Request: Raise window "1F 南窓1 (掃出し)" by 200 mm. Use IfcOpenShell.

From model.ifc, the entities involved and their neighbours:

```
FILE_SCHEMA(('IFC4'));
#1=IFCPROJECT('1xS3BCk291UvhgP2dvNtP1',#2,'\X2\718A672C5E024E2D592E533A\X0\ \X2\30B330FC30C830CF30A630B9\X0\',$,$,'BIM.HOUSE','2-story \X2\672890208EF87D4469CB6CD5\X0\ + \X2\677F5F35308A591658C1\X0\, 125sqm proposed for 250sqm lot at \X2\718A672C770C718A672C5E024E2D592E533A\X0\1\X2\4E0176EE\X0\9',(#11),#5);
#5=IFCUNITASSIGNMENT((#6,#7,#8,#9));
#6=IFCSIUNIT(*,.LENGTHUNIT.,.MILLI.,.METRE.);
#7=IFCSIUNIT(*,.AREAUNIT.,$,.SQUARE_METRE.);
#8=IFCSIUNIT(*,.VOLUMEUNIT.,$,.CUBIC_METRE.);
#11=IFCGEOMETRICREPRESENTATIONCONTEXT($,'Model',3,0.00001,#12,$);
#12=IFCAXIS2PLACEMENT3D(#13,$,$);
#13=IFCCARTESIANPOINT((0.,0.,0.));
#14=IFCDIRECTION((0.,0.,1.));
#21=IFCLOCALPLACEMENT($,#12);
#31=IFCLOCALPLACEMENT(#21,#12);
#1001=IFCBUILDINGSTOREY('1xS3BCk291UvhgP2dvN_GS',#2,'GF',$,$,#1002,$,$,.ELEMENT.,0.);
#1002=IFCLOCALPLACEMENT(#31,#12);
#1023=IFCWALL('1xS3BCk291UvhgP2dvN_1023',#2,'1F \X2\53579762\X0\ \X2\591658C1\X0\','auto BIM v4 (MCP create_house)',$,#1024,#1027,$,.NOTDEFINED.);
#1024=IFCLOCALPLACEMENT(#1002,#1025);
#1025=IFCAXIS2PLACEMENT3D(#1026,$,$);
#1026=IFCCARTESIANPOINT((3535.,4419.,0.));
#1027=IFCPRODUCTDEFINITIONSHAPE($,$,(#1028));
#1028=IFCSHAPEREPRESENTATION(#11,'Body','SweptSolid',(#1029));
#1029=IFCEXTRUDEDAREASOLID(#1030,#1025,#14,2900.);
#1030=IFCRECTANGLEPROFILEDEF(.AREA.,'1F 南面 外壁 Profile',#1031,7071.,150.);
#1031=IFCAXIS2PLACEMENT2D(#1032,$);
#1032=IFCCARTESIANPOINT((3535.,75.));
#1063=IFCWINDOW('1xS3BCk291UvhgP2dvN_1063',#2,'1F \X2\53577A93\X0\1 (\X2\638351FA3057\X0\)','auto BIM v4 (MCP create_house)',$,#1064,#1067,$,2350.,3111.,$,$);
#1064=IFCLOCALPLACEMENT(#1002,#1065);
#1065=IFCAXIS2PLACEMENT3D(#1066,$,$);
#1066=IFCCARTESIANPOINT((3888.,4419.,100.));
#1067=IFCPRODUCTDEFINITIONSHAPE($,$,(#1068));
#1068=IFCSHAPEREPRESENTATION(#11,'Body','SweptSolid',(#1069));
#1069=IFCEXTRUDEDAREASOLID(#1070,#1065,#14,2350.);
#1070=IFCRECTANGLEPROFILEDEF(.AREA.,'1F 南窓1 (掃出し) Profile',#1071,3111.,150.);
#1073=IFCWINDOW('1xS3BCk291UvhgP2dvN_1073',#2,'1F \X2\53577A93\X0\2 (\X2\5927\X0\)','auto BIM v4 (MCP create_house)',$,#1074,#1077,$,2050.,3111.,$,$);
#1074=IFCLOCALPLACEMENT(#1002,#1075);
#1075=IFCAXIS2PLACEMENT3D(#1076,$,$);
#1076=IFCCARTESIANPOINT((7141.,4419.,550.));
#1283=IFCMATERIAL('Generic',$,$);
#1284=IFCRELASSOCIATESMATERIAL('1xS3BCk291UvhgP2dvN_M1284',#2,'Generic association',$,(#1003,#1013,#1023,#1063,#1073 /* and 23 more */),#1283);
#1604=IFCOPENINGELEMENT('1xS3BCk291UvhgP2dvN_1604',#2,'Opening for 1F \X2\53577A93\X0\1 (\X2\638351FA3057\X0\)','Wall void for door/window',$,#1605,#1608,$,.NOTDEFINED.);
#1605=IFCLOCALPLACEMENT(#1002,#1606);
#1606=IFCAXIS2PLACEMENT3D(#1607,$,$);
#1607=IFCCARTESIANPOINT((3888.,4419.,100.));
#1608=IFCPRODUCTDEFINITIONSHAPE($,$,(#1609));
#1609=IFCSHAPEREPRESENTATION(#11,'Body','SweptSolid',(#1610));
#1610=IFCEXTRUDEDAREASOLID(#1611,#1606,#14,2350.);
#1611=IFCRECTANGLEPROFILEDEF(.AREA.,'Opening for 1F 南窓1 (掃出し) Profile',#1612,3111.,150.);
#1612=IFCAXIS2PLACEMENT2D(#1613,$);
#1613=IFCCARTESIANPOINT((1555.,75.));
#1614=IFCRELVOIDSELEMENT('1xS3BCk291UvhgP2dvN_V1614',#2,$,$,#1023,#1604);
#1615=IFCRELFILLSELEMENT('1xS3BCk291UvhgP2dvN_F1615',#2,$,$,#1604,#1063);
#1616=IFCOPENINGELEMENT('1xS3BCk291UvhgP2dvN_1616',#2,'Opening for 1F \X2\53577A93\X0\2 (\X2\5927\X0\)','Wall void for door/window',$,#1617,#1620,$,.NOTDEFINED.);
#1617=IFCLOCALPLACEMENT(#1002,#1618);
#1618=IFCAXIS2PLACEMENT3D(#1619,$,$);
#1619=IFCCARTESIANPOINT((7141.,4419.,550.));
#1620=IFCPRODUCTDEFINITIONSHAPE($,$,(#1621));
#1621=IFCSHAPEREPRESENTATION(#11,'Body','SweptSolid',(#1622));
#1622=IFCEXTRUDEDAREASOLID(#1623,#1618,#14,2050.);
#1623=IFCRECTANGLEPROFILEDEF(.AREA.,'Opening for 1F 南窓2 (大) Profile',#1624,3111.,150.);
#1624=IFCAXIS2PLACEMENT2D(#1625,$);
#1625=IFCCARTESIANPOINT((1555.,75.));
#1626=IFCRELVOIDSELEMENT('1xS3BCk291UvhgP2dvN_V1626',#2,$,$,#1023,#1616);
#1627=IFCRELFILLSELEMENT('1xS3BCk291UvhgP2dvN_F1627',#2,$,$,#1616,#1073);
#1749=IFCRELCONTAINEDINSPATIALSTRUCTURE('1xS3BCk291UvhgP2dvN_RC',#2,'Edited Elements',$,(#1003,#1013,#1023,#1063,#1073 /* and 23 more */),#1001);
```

```python
import numpy as np
import ifcopenshell
import ifcopenshell.api.geometry
import ifcopenshell.util.placement
import ifcopenshell.util.unit

model = ifcopenshell.open("model.ifc")
unit_scale = ifcopenshell.util.unit.calculate_unit_scale(model)

window = model.by_guid("1xS3BCk291UvhgP2dvN_1063")
opening = window.FillsVoids[0].RelatingOpeningElement
dz = 200.0

shift = np.array([0.0, 0.0, dz])
# The window is not placed relative to its opening, so move both.
for product in (opening, window):
    matrix = ifcopenshell.util.placement.get_local_placement(product.ObjectPlacement)
    matrix[:3, 3] += shift
    ifcopenshell.api.geometry.edit_object_placement(model, product=product, matrix=matrix, is_si=False)

print(f"moved by {dz * unit_scale:+.3f} m")

model.write("model_updated.ifc")
```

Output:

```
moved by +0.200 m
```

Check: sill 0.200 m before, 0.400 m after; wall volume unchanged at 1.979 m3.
